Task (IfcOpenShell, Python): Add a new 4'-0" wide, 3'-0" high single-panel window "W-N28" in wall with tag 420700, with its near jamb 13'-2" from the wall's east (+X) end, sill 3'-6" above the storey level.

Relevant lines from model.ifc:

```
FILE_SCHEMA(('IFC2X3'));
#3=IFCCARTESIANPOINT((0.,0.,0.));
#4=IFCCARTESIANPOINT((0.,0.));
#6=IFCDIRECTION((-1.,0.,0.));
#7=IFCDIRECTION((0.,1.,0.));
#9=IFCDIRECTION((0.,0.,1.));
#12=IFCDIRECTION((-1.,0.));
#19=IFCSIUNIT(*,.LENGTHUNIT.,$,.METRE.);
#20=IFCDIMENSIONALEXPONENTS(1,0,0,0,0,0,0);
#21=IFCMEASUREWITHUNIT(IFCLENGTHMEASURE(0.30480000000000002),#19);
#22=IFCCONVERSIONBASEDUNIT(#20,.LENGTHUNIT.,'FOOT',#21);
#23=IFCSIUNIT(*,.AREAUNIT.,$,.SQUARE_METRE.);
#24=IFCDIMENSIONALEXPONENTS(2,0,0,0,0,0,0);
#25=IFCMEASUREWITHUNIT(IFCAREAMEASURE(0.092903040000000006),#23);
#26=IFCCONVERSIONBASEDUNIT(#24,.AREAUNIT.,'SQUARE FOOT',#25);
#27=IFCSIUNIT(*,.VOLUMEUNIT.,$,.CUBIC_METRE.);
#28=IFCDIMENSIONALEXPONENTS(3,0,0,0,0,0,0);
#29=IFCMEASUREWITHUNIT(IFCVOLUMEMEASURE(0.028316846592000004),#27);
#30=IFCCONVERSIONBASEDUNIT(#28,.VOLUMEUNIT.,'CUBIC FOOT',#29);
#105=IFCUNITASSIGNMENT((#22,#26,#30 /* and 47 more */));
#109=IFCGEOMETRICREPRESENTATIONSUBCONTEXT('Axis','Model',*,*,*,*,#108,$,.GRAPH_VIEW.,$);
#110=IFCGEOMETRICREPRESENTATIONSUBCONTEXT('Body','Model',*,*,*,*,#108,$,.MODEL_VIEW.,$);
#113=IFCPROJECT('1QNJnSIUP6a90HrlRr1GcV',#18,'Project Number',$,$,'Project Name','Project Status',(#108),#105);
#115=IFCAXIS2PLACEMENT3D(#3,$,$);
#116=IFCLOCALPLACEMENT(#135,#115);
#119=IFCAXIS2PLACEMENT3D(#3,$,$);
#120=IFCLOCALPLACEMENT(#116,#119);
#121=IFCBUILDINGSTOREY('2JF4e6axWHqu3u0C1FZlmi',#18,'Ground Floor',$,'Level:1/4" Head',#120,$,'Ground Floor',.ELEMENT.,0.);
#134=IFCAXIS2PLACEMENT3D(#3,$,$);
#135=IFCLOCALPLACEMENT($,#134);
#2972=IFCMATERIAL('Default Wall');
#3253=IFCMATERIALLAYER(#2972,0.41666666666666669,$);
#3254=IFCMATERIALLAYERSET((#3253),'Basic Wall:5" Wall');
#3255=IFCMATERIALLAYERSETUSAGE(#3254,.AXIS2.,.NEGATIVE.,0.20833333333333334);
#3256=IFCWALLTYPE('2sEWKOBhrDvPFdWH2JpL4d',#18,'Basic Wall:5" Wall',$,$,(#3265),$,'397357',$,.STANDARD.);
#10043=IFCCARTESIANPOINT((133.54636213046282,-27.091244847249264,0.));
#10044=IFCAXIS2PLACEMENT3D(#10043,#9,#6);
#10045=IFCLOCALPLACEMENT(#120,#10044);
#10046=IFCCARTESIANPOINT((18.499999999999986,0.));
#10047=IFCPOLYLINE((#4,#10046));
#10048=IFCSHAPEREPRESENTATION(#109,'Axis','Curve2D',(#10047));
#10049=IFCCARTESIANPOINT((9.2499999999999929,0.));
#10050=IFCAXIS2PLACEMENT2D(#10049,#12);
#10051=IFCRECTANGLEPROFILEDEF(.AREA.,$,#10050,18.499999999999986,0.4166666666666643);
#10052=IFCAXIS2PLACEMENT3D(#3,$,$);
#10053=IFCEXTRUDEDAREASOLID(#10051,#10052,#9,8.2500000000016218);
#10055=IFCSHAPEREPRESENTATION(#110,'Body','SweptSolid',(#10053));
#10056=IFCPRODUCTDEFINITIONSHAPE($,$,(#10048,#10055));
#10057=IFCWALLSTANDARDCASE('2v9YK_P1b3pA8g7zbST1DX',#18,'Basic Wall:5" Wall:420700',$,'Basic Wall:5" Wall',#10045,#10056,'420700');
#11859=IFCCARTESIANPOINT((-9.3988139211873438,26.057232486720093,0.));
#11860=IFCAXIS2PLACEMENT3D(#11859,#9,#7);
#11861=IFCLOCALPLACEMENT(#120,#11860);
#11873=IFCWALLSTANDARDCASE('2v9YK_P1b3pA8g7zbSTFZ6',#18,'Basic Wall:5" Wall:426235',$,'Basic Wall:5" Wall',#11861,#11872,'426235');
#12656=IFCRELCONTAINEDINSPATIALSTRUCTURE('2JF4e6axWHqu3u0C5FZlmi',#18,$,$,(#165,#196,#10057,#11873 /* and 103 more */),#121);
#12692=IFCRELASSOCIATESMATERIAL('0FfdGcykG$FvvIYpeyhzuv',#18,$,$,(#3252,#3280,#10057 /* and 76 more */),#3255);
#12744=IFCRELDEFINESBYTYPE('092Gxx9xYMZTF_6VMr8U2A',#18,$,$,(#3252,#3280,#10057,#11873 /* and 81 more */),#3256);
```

```python
import numpy as np
import ifcopenshell
import ifcopenshell.api.feature
import ifcopenshell.api.geometry
import ifcopenshell.api.root
import ifcopenshell.api.spatial
import ifcopenshell.api.type
import ifcopenshell.geom
import ifcopenshell.util.element
import ifcopenshell.util.placement
import ifcopenshell.util.representation
import ifcopenshell.util.shape
import ifcopenshell.util.unit

model = ifcopenshell.open("model.ifc")
unit_scale = ifcopenshell.util.unit.calculate_unit_scale(model)
settings = ifcopenshell.geom.settings()


def volume(element):
    """Net volume in cubic metres, openings subtracted."""
    shape = ifcopenshell.geom.create_shape(settings, element)
    return ifcopenshell.util.shape.get_volume(shape.geometry)


wall = model.by_id(10057)
storey = ifcopenshell.util.element.get_container(wall, ifc_class="IfcBuildingStorey")
context = ifcopenshell.util.representation.get_context(model, "Model", "Body", "MODEL_VIEW")
before = volume(wall)

width, height, from_end, sill = 1.2192, 0.9144, 4.0132, 1.0668  # metres

# The wall runs along its own X axis, and the end named is its -X end.
wall_shape = ifcopenshell.geom.create_shape(settings, wall)
x, y, z = ifcopenshell.util.shape.get_vertices(wall_shape.geometry).T
start = x.min() + from_end
face, thickness = float(y.min()), float(y.max() - y.min())
wall_matrix = ifcopenshell.util.placement.get_local_placement(wall.ObjectPlacement)
level = ifcopenshell.util.placement.get_local_placement(storey.ObjectPlacement)[2, 3]


def in_wall(x, y):
    """Placement at x, y metres in the wall's axes, at sill height."""
    matrix = wall_matrix.copy()
    matrix[:, 3] = wall_matrix @ np.array([x / unit_scale, y / unit_scale, 0.0, 1.0])
    matrix[2, 3] = level + sill / unit_scale
    return matrix


# Opening: a box that overshoots both wall faces by 50 mm.
opening = ifcopenshell.api.root.create_entity(model, ifc_class="IfcOpeningElement")
box = ifcopenshell.api.geometry.add_wall_representation(
    model, context=context, length=width, height=height, thickness=thickness + 0.1
)
ifcopenshell.api.geometry.assign_representation(model, product=opening, representation=box)
ifcopenshell.api.geometry.edit_object_placement(model, product=opening, matrix=in_wall(start, face - 0.05), is_si=False)
ifcopenshell.api.feature.add_feature(model, feature=opening, element=wall)

window = ifcopenshell.api.root.create_entity(model, ifc_class="IfcWindow", name="W-N28")
window.OverallWidth, window.OverallHeight = width / unit_scale, height / unit_scale
body = ifcopenshell.api.geometry.add_window_representation(
    model,
    context=context,
    overall_width=window.OverallWidth,
    overall_height=window.OverallHeight,
    partition_type="SINGLE_PANEL",
)
ifcopenshell.api.geometry.assign_representation(model, product=window, representation=body)
ifcopenshell.api.spatial.assign_container(model, products=[window], relating_structure=storey)
fills = ifcopenshell.api.feature.add_filling(model, opening=opening, element=window)
fills.OwnerHistory = window.OwnerHistory  # required in IFC2X3

# IFC2X3 keeps the operation on the window style.
style = ifcopenshell.api.root.create_entity(model, ifc_class="IfcWindowStyle", name="W-N28")
style.OperationType, style.ConstructionType = "SINGLE_PANEL", "NOTDEFINED"
style.ParameterTakesPrecedence = style.Sizeable = False
ifcopenshell.api.type.assign_type(model, related_objects=[window], relating_type=style)

# Centre the window in the wall's thickness.
ifcopenshell.api.geometry.edit_object_placement(model, product=window, matrix=in_wall(start, face), is_si=False)
window_shape = ifcopenshell.geom.create_shape(settings, window)
depth = ifcopenshell.util.shape.get_vertices(window_shape.geometry)[:, 1]
offset = face + thickness / 2 - (depth.min() + depth.max()) / 2
ifcopenshell.api.geometry.edit_object_placement(model, product=window, matrix=in_wall(start, offset), is_si=False)

after = volume(wall)

print(f"wall volume {before:.3f} -> {after:.3f} m3")

model.write("model_edited.ifc")
```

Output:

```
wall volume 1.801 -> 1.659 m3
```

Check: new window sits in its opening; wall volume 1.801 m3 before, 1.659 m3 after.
